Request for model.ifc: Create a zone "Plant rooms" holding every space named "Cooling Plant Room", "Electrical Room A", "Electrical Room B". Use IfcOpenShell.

First a look at what the model holds.

```python
import ifcopenshell

model = ifcopenshell.open("model.ifc")
print(model.schema)
seen = {}
for space in model.by_type("IfcSpace"):
    seen[space.LongName] = seen.get(space.LongName, 0) + 1
for name, count in sorted(seen.items(), key=str):
    print(count, "x", name)
print("zones:", [z.Name for z in model.by_type("IfcZone")][:20])
```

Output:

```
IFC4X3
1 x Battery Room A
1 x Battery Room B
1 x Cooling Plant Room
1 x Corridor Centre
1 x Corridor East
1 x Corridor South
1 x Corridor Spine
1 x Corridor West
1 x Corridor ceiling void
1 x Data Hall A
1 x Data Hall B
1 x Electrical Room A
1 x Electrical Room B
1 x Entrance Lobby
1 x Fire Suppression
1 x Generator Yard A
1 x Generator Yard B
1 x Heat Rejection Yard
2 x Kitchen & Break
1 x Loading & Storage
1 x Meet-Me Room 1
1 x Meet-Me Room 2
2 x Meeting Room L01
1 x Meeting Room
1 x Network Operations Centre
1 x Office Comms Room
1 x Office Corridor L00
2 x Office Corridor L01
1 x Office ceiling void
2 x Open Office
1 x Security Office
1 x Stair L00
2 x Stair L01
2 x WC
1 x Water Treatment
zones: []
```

```python
import ifcopenshell
import ifcopenshell.api.group
import ifcopenshell.api.root

model = ifcopenshell.open("model.ifc")

names = {"Cooling Plant Room", "Electrical Room A", "Electrical Room B"}
spaces = [s for s in model.by_type("IfcSpace") if s.LongName in names]

zone = ifcopenshell.api.root.create_entity(model, ifc_class="IfcZone", name="Plant rooms")
ifcopenshell.api.group.assign_group(model, products=spaces, group=zone)
print(len(spaces), "spaces in", zone.Name)

model.write("model_rev.ifc")
```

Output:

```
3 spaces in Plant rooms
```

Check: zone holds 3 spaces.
